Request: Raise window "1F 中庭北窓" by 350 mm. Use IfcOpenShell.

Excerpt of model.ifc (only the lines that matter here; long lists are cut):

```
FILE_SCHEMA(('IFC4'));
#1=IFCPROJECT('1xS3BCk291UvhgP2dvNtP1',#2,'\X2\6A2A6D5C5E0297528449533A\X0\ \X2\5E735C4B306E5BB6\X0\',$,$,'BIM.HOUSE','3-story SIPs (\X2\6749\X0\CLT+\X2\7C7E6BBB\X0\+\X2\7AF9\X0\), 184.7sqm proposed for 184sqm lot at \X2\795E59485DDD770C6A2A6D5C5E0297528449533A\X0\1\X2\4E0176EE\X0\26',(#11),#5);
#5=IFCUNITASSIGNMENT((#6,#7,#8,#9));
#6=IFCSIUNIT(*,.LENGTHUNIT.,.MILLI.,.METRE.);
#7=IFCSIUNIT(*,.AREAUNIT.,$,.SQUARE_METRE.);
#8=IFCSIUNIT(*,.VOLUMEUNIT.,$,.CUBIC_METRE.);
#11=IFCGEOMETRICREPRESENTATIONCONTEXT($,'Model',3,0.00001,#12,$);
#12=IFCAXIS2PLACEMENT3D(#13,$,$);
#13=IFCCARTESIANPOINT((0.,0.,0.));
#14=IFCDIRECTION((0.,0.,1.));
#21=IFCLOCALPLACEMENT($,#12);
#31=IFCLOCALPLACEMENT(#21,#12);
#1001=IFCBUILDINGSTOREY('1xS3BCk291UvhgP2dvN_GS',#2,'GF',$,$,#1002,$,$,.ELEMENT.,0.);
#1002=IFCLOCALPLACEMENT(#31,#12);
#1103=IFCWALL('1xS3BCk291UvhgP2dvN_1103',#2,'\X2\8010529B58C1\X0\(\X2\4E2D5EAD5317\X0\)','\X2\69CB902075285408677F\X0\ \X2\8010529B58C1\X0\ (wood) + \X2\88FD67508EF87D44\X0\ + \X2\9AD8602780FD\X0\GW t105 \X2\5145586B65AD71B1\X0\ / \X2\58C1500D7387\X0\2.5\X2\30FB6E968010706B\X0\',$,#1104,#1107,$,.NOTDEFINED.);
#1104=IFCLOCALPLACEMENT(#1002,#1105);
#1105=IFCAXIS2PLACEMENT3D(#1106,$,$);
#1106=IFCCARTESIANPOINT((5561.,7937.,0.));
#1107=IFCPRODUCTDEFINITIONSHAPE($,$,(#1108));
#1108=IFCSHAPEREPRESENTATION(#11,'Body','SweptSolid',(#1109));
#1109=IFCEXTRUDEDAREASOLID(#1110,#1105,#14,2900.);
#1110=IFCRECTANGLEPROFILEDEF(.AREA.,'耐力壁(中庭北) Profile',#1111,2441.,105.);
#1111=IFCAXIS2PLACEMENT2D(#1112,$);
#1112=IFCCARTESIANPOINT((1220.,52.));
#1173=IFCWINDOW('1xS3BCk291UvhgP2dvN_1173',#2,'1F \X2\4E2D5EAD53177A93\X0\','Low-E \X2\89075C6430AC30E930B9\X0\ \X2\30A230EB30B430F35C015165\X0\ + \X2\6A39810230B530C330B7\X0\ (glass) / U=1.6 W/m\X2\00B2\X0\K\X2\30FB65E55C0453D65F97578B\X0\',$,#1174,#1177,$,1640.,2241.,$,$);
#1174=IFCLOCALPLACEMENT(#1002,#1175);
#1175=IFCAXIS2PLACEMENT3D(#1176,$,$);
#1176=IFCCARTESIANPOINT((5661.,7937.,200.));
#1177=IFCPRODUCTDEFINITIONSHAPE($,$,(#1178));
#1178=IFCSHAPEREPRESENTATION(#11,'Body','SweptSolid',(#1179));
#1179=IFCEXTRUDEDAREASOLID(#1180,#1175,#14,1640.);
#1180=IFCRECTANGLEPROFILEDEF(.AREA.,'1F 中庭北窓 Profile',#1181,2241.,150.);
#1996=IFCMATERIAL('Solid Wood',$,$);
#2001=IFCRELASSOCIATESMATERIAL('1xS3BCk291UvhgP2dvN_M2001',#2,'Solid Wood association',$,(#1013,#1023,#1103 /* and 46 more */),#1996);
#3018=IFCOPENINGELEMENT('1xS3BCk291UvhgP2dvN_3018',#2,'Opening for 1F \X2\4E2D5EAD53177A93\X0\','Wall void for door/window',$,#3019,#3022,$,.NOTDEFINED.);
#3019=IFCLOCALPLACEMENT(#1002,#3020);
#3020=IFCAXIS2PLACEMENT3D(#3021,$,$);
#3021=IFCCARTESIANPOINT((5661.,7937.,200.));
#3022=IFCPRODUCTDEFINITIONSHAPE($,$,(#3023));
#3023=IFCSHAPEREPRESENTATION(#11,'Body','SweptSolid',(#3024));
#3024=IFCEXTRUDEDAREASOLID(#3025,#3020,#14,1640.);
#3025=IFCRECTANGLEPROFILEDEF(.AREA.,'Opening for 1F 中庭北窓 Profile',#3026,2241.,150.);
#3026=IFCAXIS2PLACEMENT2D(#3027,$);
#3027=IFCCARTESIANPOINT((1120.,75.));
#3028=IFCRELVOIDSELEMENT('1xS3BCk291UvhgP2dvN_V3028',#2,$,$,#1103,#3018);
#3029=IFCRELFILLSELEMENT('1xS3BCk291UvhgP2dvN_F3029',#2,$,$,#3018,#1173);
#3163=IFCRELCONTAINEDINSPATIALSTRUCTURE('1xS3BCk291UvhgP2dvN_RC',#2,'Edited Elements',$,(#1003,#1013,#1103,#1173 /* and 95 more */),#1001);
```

```python
import numpy as np
import ifcopenshell
import ifcopenshell.api.geometry
import ifcopenshell.util.placement
import ifcopenshell.util.unit

model = ifcopenshell.open("model.ifc")
unit_scale = ifcopenshell.util.unit.calculate_unit_scale(model)

window = model.by_guid("1xS3BCk291UvhgP2dvN_1173")
opening = window.FillsVoids[0].RelatingOpeningElement
dz = 350.0

shift = np.array([0.0, 0.0, dz])
# The window is not placed relative to its opening, so move both.
for product in (opening, window):
    matrix = ifcopenshell.util.placement.get_local_placement(product.ObjectPlacement)
    matrix[:3, 3] += shift
    ifcopenshell.api.geometry.edit_object_placement(model, product=product, matrix=matrix, is_si=False)

print(f"moved by {dz * unit_scale:+.3f} m")

model.write("model_edited.ifc")
```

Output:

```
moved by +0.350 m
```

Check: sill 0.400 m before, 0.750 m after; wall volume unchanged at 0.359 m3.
